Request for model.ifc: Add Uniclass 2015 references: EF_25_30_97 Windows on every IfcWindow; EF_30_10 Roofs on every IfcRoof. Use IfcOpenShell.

First a look at what the model holds.

```python
import ifcopenshell

model = ifcopenshell.open("model.ifc")
print(model.schema)
print("classifications:", [c.Name for c in model.by_type("IfcClassification")])
for ifc_class in ("IfcDoor", "IfcRoof", "IfcStair", "IfcWall", "IfcWindow"):
    print(ifc_class, len(model.by_type(ifc_class)))
```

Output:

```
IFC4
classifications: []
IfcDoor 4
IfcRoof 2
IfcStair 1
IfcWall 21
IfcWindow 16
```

```python
import ifcopenshell
import ifcopenshell.api.classification

model = ifcopenshell.open("model.ifc")

system = ifcopenshell.api.classification.add_classification(model, classification="Uniclass 2015")

codes = {
    "IfcWindow": ("EF_25_30_97", "Windows"),
    "IfcRoof": ("EF_30_10", "Roofs"),
}
for ifc_class, (code, name) in codes.items():
    products = model.by_type(ifc_class)
    ifcopenshell.api.classification.add_reference(
        model, products=products, classification=system, identification=code, name=name
    )
    print(code, len(products))

model.write("model-out.ifc")
```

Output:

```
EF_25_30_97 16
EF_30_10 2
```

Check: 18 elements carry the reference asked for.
